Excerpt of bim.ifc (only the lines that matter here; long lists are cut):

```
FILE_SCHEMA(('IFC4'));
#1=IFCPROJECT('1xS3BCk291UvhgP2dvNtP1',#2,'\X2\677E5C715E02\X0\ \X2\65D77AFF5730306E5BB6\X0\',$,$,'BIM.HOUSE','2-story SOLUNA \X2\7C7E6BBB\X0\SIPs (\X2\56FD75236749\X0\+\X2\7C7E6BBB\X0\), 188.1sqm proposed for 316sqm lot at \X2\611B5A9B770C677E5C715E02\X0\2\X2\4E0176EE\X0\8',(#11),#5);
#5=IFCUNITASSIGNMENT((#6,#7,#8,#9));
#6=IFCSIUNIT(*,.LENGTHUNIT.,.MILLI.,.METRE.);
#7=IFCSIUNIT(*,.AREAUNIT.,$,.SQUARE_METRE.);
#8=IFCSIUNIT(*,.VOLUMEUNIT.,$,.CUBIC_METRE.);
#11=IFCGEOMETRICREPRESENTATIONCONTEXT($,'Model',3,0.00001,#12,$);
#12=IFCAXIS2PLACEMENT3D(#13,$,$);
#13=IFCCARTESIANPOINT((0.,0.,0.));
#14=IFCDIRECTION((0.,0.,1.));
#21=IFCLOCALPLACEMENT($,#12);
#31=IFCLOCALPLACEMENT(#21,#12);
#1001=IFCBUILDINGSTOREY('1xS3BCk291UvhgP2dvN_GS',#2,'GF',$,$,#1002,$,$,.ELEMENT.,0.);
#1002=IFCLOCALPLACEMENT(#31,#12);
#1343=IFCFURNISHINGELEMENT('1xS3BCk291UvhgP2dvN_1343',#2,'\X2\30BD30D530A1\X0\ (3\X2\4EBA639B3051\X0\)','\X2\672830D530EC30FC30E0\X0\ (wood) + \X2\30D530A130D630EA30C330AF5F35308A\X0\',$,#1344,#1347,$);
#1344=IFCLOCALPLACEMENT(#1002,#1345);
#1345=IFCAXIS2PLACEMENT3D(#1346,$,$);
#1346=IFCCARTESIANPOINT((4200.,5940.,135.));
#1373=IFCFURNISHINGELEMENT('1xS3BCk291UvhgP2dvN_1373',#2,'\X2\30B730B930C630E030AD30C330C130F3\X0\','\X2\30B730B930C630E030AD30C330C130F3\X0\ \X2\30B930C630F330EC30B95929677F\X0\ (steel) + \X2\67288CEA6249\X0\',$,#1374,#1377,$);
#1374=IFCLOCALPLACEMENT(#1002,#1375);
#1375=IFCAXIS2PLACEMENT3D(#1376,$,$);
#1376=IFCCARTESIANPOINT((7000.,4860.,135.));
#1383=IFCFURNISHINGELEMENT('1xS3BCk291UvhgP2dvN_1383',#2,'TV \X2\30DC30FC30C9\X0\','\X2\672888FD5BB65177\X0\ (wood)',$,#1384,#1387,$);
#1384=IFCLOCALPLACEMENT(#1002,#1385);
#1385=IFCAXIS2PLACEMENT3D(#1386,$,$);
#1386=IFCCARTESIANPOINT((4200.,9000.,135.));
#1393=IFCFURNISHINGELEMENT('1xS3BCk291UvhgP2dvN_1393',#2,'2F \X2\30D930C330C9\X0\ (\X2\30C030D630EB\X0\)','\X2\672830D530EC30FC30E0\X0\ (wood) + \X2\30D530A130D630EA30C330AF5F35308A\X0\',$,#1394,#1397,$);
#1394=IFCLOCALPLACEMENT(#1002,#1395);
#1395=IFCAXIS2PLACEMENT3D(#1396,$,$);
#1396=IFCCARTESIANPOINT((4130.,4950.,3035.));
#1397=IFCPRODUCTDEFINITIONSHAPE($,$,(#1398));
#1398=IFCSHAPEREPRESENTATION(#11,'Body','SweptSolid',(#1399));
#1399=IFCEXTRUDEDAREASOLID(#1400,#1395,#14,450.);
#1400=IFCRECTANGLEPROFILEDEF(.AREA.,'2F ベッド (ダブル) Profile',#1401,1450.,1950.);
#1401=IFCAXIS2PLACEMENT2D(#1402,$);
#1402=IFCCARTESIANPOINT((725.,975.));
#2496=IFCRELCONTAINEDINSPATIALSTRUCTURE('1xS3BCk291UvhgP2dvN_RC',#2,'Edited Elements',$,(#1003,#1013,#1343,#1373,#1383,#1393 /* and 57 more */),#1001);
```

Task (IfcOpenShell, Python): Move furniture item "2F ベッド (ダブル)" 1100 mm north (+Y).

```python
import ifcopenshell
import ifcopenshell.api.geometry
import ifcopenshell.util.placement

model = ifcopenshell.open("bim.ifc")

item = model.by_guid("1xS3BCk291UvhgP2dvN_1393")
matrix = ifcopenshell.util.placement.get_local_placement(item.ObjectPlacement)
matrix[1, 3] += 1100.0
ifcopenshell.api.geometry.edit_object_placement(model, product=item, matrix=matrix, is_si=False)

print(ifcopenshell.util.placement.get_local_placement(item.ObjectPlacement).round(3) + 0.0)

model.write("bim_updated.ifc")
```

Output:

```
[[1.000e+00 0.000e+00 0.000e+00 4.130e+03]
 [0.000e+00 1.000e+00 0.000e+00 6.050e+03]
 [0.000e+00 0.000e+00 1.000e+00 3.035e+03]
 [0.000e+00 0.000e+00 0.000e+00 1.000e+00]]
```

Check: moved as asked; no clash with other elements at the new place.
